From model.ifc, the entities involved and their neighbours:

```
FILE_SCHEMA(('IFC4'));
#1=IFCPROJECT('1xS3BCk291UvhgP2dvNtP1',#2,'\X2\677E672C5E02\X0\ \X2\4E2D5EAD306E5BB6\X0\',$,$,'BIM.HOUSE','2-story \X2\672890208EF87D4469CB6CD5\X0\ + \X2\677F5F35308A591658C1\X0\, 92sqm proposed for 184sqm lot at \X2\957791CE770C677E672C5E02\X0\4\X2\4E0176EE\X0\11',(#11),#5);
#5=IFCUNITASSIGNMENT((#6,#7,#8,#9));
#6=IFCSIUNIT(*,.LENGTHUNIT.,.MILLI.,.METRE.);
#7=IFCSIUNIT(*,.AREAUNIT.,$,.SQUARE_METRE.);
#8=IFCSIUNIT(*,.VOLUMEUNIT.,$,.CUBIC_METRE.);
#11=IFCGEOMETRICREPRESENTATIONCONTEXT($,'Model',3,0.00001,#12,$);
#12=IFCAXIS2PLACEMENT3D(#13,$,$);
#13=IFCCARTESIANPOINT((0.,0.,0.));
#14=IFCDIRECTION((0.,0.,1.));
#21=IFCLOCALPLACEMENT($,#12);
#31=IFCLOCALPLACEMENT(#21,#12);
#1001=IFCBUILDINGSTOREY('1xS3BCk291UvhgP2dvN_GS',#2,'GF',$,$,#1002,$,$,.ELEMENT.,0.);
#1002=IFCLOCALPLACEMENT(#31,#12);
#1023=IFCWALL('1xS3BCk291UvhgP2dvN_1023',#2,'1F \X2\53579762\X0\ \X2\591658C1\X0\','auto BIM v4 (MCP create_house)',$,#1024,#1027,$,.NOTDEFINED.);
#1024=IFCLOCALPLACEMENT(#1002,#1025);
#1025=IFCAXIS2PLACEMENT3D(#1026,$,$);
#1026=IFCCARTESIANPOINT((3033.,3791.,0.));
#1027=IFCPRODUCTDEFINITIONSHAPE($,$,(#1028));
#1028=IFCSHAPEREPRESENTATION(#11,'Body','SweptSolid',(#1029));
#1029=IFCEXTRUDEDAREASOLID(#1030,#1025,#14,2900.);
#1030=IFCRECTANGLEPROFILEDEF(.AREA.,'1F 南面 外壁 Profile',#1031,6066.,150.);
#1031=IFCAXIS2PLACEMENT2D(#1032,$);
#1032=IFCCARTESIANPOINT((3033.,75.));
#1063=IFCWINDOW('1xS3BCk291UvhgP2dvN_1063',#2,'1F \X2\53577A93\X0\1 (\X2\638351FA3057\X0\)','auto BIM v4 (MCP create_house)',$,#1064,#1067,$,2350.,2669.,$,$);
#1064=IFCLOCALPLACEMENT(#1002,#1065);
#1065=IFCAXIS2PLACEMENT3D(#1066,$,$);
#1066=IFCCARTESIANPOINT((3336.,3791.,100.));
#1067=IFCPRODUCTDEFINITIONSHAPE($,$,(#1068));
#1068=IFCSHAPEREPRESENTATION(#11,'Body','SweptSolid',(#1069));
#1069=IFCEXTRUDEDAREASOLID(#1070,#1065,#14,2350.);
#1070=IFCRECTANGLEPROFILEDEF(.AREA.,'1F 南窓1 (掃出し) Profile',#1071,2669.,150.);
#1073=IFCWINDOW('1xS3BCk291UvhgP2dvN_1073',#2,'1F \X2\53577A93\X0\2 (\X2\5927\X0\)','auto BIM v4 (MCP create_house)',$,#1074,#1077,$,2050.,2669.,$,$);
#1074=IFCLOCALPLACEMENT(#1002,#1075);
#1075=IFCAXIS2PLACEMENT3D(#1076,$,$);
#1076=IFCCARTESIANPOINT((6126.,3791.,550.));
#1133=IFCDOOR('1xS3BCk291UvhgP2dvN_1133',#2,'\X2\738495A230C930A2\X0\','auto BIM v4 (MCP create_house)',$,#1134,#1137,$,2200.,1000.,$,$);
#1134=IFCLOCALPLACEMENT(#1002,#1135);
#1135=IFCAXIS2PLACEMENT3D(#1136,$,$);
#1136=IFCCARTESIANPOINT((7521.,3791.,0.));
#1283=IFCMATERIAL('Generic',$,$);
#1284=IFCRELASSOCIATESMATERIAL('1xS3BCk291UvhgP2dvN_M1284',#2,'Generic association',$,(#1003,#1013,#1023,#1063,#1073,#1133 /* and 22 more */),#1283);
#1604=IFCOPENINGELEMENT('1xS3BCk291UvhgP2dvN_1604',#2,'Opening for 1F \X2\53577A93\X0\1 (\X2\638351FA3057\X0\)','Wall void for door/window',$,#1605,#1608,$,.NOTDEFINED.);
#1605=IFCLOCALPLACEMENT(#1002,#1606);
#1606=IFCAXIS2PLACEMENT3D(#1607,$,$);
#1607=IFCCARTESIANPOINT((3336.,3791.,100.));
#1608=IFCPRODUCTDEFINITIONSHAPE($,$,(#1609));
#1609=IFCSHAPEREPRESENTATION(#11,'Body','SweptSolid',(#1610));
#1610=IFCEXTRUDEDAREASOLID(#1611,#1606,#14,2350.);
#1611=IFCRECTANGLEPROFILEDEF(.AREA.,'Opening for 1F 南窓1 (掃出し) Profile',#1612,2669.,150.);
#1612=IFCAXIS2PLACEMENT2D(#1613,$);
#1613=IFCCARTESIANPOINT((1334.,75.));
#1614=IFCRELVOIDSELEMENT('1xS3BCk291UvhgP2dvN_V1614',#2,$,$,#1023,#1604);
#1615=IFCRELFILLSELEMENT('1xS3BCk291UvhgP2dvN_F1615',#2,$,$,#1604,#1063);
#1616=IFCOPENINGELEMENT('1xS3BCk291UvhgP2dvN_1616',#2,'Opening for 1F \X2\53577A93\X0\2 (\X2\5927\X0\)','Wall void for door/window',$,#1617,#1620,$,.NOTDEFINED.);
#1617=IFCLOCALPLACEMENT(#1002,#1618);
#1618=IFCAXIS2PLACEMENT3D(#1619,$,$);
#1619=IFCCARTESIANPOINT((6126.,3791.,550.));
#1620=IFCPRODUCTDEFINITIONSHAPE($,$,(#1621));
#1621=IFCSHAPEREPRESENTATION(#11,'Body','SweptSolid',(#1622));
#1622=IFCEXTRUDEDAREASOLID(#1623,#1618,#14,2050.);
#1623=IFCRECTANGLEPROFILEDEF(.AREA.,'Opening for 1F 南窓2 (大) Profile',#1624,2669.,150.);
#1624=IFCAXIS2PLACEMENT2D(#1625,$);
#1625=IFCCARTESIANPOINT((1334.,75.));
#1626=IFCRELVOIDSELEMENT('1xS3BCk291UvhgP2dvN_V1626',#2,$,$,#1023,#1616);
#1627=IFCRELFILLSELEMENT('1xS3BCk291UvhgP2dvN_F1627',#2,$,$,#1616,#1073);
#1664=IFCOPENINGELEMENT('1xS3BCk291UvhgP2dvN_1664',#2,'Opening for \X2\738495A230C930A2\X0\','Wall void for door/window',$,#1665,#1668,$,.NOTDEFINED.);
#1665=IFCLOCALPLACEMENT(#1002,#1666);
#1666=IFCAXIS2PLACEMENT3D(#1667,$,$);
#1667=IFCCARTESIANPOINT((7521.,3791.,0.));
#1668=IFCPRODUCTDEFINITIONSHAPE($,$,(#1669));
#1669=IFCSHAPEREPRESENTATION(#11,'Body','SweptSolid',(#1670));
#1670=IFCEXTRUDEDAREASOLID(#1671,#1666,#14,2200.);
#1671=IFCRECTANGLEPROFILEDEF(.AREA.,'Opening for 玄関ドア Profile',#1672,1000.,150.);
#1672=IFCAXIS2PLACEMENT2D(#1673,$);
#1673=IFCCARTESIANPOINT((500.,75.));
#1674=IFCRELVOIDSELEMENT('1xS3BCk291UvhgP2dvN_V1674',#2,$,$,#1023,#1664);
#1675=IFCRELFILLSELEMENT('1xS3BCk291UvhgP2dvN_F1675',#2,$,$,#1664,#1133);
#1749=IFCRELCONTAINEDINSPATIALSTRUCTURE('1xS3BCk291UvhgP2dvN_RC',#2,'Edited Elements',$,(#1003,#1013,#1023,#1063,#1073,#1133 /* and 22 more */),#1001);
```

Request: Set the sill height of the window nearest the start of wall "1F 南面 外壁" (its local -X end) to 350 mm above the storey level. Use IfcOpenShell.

```python
import numpy as np
import ifcopenshell
import ifcopenshell.api.geometry
import ifcopenshell.geom
import ifcopenshell.util.element
import ifcopenshell.util.placement
import ifcopenshell.util.shape
import ifcopenshell.util.unit

model = ifcopenshell.open("model.ifc")
unit_scale = ifcopenshell.util.unit.calculate_unit_scale(model)

window = model.by_id(1063)
opening = window.FillsVoids[0].RelatingOpeningElement
storey = ifcopenshell.util.element.get_container(window, ifc_class="IfcBuildingStorey")
level = ifcopenshell.util.placement.get_local_placement(storey.ObjectPlacement)[2, 3]

# The opening's origin need not be at the sill, so measure its lowest point.
shape = ifcopenshell.geom.create_shape(ifcopenshell.geom.settings(), opening)
bottom = ifcopenshell.util.shape.get_shape_bottom_elevation(shape, shape.geometry) / unit_scale
dz = level + 350.0 - bottom

shift = np.array([0.0, 0.0, dz])
# The window is not placed relative to its opening, so move both.
for product in (opening, window):
    matrix = ifcopenshell.util.placement.get_local_placement(product.ObjectPlacement)
    matrix[:3, 3] += shift
    ifcopenshell.api.geometry.edit_object_placement(model, product=product, matrix=matrix, is_si=False)

print(f"moved by {dz * unit_scale:+.3f} m")

model.write("model_v2.ifc")
```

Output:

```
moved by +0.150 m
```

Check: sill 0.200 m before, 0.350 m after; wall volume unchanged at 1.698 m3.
